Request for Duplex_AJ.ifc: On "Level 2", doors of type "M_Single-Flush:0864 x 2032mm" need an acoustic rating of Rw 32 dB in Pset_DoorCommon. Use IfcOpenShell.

First a look at what the model holds.

```python
import ifcopenshell
import ifcopenshell.util.element

model = ifcopenshell.open("Duplex_AJ.ifc")
print(model.schema)
storey = next(s for s in model.by_type("IfcBuildingStorey") if s.Name == "Level 2")
doors = [e for e in ifcopenshell.util.element.get_decomposition(storey) if e.is_a("IfcDoor")]
seen = {}
for e in doors:
    element_type = ifcopenshell.util.element.get_type(e)
    key = (element_type.Name if element_type != e and element_type else None, ifcopenshell.util.element.get_pset(e, "Pset_DoorCommon", "AcousticRating"))
    seen[key] = seen.get(key, 0) + 1
for (name, value), count in sorted(seen.items(), key=str):
    print(count, "x", name, "|", value)
```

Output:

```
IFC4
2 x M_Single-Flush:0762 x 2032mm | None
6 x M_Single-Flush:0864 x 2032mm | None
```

```python
import ifcopenshell
import ifcopenshell.api.pset
import ifcopenshell.util.element

model = ifcopenshell.open("Duplex_AJ.ifc")

storey = next(s for s in model.by_type("IfcBuildingStorey") if s.Name == "Level 2")
doors = [e for e in ifcopenshell.util.element.get_decomposition(storey) if e.is_a("IfcDoor")]

count = 0
for e in doors:
    element_type = ifcopenshell.util.element.get_type(e)
    if element_type in (None, e) or element_type.Name != "M_Single-Flush:0864 x 2032mm":
        continue
    # add_pset returns the element's existing set when there is one.
    pset = ifcopenshell.api.pset.add_pset(model, product=e, name="Pset_DoorCommon")
    ifcopenshell.api.pset.edit_pset(model, pset=pset, properties={"AcousticRating": "Rw 32 dB"})
    count += 1

print(count, "doors updated")

model.write("Duplex_AJ_updated.ifc")
```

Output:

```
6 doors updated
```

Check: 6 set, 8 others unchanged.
